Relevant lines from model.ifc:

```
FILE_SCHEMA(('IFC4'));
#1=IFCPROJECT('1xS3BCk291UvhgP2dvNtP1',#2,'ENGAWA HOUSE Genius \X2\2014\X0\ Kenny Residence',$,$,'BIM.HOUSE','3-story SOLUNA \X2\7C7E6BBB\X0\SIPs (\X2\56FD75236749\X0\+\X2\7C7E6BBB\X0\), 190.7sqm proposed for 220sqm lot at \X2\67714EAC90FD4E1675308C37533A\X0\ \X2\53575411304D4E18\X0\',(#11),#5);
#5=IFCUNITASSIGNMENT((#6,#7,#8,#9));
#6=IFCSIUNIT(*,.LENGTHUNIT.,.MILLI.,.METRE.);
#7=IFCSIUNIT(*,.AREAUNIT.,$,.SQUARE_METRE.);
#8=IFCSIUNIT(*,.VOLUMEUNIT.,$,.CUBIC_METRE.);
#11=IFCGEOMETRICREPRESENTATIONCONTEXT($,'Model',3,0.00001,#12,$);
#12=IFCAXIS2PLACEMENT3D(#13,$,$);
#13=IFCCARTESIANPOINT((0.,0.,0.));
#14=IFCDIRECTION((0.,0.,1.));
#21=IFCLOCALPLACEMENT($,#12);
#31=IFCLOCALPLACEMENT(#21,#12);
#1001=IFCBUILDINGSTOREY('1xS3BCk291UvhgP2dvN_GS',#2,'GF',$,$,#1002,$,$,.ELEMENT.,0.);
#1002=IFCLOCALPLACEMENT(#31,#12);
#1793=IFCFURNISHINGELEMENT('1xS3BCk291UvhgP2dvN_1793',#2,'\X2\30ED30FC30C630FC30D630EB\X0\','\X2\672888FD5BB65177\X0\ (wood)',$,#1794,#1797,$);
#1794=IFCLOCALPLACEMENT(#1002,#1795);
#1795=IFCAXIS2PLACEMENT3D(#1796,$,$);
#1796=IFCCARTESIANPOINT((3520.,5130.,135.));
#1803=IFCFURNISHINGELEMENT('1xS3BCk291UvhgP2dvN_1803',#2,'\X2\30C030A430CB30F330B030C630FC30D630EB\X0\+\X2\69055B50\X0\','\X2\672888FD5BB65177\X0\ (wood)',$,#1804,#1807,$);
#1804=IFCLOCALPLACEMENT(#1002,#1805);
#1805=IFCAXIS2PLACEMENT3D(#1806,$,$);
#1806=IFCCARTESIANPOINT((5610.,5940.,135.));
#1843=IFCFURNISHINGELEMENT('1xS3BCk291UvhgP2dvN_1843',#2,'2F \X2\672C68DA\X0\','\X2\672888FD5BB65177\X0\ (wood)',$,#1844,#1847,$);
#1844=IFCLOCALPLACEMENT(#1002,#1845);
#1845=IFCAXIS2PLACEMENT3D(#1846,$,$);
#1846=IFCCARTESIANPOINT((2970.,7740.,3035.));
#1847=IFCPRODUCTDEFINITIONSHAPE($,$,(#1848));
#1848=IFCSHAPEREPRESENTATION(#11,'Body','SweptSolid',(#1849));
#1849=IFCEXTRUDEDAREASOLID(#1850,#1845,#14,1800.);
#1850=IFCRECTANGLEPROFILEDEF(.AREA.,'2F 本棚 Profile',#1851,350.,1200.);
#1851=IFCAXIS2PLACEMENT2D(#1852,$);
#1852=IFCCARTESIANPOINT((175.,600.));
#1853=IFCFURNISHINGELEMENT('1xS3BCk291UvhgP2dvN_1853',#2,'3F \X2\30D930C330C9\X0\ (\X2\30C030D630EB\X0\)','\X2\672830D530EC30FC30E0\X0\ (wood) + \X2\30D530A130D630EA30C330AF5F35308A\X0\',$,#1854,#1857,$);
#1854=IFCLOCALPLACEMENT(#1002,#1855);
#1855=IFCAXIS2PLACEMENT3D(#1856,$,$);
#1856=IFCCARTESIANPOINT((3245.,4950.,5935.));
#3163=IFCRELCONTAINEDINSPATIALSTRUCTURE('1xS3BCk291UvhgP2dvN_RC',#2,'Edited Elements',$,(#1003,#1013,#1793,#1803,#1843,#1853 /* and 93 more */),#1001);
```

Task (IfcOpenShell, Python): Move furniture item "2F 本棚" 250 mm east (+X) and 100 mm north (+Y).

```python
import ifcopenshell
import ifcopenshell.api.geometry
import ifcopenshell.util.placement

model = ifcopenshell.open("model.ifc")

item = model.by_guid("1xS3BCk291UvhgP2dvN_1843")
matrix = ifcopenshell.util.placement.get_local_placement(item.ObjectPlacement)
matrix[0, 3] += 250.0
matrix[1, 3] += 100.0
ifcopenshell.api.geometry.edit_object_placement(model, product=item, matrix=matrix, is_si=False)

print(ifcopenshell.util.placement.get_local_placement(item.ObjectPlacement).round(3) + 0.0)

model.write("model_v2.ifc")
```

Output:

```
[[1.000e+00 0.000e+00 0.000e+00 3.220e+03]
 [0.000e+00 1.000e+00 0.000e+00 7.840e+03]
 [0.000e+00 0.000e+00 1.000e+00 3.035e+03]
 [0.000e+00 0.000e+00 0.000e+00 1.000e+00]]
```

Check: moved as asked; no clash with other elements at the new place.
